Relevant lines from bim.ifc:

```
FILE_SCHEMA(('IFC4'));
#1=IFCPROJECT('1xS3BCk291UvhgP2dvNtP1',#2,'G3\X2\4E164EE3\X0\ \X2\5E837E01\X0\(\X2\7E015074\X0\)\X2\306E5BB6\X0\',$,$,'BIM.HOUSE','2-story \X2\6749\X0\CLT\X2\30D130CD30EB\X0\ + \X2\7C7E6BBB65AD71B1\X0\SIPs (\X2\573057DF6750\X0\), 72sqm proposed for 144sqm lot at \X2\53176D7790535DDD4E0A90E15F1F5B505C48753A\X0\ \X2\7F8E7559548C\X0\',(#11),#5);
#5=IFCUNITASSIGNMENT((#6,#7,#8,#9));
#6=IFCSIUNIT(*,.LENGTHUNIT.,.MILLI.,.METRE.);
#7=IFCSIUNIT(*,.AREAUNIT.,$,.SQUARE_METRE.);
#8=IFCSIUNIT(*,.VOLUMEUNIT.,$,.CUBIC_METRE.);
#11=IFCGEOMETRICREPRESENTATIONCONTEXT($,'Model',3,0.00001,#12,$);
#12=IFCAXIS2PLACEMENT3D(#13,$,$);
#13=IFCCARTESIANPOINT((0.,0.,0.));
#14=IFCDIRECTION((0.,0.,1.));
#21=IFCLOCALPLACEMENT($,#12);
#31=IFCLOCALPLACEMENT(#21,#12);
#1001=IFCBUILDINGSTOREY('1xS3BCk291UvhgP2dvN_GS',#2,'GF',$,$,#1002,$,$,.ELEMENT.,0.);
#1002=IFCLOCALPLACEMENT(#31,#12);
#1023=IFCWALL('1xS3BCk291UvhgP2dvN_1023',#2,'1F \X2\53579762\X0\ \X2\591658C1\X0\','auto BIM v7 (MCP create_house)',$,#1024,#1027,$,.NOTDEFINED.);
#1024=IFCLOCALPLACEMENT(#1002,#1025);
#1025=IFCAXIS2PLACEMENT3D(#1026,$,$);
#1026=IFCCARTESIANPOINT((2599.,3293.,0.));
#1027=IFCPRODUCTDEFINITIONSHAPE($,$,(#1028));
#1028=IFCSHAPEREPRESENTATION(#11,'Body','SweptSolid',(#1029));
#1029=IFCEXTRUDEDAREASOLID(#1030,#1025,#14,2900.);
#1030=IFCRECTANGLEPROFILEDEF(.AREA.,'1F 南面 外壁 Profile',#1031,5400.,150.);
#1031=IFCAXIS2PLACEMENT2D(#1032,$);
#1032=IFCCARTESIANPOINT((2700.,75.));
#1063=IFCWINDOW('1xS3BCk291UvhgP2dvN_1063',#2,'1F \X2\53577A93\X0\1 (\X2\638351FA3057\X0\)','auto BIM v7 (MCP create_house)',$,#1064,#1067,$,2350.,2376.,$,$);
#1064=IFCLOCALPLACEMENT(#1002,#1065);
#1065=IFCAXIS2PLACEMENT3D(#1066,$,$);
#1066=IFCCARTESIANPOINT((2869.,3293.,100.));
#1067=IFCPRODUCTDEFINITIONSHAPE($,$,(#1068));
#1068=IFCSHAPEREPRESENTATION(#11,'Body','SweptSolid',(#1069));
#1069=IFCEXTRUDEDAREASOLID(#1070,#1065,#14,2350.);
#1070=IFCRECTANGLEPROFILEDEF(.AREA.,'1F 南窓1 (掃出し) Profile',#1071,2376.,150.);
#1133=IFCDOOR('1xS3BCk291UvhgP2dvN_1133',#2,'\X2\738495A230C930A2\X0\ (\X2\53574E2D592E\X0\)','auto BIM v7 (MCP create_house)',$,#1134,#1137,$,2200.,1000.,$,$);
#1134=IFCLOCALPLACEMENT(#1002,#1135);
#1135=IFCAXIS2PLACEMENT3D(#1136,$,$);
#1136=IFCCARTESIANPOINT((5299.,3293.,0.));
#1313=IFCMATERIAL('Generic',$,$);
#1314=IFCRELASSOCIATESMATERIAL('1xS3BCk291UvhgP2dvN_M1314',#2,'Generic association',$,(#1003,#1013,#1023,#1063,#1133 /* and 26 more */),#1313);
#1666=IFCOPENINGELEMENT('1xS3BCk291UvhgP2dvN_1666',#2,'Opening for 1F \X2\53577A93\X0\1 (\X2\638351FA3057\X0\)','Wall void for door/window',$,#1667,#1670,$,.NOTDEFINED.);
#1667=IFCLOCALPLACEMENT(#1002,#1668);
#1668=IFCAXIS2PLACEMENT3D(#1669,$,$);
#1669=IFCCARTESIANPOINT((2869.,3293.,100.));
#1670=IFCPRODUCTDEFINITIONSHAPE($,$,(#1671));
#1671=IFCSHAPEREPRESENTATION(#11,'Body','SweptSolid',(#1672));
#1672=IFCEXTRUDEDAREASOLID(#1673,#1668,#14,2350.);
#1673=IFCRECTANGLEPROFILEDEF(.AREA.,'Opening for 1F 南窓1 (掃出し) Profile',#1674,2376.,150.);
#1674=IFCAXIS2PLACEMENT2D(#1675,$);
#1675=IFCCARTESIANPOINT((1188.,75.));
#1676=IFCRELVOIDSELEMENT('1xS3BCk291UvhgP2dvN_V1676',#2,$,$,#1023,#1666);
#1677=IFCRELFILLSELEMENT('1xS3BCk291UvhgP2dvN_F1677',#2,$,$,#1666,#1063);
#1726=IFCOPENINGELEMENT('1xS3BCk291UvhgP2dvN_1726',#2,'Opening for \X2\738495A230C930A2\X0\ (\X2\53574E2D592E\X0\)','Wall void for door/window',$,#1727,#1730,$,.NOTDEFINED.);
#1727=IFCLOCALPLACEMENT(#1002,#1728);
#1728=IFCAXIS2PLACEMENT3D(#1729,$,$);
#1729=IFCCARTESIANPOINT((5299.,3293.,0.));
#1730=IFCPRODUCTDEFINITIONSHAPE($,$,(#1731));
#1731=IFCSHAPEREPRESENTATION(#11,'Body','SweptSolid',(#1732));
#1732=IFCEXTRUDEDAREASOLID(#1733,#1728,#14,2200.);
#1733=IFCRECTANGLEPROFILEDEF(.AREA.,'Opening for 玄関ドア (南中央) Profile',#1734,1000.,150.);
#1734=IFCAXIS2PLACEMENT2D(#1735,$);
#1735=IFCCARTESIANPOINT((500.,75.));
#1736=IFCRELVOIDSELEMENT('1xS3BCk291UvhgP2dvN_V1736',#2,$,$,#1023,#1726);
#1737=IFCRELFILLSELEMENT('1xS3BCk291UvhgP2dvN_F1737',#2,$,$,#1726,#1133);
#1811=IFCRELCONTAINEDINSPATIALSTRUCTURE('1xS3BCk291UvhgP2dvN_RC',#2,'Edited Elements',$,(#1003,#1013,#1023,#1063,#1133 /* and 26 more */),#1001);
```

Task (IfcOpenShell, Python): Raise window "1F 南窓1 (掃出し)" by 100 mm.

```python
import numpy as np
import ifcopenshell
import ifcopenshell.api.geometry
import ifcopenshell.util.placement
import ifcopenshell.util.unit

model = ifcopenshell.open("bim.ifc")
unit_scale = ifcopenshell.util.unit.calculate_unit_scale(model)

window = model.by_guid("1xS3BCk291UvhgP2dvN_1063")
opening = window.FillsVoids[0].RelatingOpeningElement
dz = 0.1 / unit_scale

shift = np.array([0.0, 0.0, dz])
# The window is not placed relative to its opening, so move both.
for product in (opening, window):
    matrix = ifcopenshell.util.placement.get_local_placement(product.ObjectPlacement)
    matrix[:3, 3] += shift
    ifcopenshell.api.geometry.edit_object_placement(model, product=product, matrix=matrix, is_si=False)

print(f"moved by {dz * unit_scale:+.3f} m")

model.write("bim_edited.ifc")
```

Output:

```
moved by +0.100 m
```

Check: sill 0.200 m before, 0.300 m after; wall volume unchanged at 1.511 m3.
